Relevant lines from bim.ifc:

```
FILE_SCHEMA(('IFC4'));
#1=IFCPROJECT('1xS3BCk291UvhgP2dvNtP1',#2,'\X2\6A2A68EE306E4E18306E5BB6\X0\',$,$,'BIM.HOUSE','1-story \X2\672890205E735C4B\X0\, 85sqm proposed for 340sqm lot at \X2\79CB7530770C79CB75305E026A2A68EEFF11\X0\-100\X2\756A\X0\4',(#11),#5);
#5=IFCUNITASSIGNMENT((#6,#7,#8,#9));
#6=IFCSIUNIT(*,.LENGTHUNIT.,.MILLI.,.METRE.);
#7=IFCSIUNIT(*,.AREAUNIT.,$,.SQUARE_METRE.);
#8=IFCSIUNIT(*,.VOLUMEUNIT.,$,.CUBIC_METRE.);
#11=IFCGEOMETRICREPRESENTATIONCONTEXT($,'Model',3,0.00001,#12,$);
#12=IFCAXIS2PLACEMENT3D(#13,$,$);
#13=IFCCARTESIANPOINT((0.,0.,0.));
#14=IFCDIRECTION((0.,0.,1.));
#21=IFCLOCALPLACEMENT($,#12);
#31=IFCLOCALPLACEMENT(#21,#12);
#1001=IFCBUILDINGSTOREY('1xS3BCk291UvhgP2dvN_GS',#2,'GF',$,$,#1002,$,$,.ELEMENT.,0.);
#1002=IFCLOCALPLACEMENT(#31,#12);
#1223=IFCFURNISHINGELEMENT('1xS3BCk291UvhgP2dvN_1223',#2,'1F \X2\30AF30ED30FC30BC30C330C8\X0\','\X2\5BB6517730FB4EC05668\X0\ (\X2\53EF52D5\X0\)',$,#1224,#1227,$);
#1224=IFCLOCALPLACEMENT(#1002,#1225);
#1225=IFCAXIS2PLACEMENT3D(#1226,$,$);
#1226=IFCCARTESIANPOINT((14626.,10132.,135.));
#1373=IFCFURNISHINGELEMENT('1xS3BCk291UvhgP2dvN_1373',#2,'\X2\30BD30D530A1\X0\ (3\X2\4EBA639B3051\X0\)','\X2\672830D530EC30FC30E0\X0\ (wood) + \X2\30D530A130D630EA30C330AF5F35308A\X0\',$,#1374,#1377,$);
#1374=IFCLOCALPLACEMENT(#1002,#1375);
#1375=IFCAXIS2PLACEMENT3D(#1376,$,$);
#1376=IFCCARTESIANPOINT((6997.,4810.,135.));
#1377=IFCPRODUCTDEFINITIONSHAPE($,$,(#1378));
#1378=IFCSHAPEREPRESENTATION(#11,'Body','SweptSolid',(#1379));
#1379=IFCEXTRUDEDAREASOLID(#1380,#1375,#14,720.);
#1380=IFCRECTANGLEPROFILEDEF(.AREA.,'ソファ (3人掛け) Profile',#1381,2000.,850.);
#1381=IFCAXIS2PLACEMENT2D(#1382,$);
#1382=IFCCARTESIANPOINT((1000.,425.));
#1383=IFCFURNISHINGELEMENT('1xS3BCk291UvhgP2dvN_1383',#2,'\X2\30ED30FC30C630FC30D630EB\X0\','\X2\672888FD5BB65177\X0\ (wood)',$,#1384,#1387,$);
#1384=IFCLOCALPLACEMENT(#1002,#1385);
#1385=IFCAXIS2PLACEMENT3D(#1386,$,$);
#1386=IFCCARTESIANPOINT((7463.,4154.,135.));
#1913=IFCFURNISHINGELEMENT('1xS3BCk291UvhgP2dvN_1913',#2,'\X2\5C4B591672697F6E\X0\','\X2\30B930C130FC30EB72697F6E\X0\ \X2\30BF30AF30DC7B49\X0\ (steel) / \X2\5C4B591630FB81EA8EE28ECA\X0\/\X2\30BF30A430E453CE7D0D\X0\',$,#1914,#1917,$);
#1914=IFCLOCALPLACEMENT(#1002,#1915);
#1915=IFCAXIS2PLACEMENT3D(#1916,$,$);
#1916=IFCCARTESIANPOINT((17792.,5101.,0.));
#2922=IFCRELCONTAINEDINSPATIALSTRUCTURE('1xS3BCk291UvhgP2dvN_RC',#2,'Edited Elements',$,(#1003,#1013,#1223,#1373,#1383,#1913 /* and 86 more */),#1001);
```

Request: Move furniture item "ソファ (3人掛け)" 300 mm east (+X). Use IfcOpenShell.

```python
import ifcopenshell
import ifcopenshell.api.geometry
import ifcopenshell.util.placement
import ifcopenshell.util.unit

model = ifcopenshell.open("bim.ifc")
unit_scale = ifcopenshell.util.unit.calculate_unit_scale(model)

item = model.by_guid("1xS3BCk291UvhgP2dvN_1373")
matrix = ifcopenshell.util.placement.get_local_placement(item.ObjectPlacement)
matrix[0, 3] += 0.3 / unit_scale
ifcopenshell.api.geometry.edit_object_placement(model, product=item, matrix=matrix, is_si=False)

print(ifcopenshell.util.placement.get_local_placement(item.ObjectPlacement).round(3) + 0.0)

model.write("bim_v2.ifc")
```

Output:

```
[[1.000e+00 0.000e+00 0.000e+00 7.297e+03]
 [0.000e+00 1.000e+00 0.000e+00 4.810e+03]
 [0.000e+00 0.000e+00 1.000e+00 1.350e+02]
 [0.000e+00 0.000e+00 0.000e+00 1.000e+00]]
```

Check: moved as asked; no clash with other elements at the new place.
